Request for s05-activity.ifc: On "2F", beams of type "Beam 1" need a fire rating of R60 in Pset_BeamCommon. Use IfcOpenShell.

First a look at what the model holds.

```python
import ifcopenshell
import ifcopenshell.util.element

model = ifcopenshell.open("s05-activity.ifc")
print(model.schema)
storey = next(s for s in model.by_type("IfcBuildingStorey") if s.Name == "2F")
beams = [e for e in ifcopenshell.util.element.get_decomposition(storey) if e.is_a("IfcBeam")]
seen = {}
for e in beams:
    element_type = ifcopenshell.util.element.get_type(e)
    key = (element_type.Name if element_type != e and element_type else None, ifcopenshell.util.element.get_pset(e, "Pset_BeamCommon", "FireRating"))
    seen[key] = seen.get(key, 0) + 1
for (name, value), count in sorted(seen.items(), key=str):
    print(count, "x", name, "|", value)
```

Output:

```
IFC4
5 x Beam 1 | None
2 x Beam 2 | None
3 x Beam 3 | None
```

```python
import ifcopenshell
import ifcopenshell.api.pset
import ifcopenshell.util.element

model = ifcopenshell.open("s05-activity.ifc")

storey = next(s for s in model.by_type("IfcBuildingStorey") if s.Name == "2F")
beams = [e for e in ifcopenshell.util.element.get_decomposition(storey) if e.is_a("IfcBeam")]

count = 0
for e in beams:
    element_type = ifcopenshell.util.element.get_type(e)
    if element_type in (None, e) or element_type.Name != "Beam 1":
        continue
    # add_pset returns the element's existing set when there is one.
    pset = ifcopenshell.api.pset.add_pset(model, product=e, name="Pset_BeamCommon")
    ifcopenshell.api.pset.edit_pset(model, pset=pset, properties={"FireRating": "R60"})
    count += 1

print(count, "beams updated")

model.write("s05-activity_rev.ifc")
```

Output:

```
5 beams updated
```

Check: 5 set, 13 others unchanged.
